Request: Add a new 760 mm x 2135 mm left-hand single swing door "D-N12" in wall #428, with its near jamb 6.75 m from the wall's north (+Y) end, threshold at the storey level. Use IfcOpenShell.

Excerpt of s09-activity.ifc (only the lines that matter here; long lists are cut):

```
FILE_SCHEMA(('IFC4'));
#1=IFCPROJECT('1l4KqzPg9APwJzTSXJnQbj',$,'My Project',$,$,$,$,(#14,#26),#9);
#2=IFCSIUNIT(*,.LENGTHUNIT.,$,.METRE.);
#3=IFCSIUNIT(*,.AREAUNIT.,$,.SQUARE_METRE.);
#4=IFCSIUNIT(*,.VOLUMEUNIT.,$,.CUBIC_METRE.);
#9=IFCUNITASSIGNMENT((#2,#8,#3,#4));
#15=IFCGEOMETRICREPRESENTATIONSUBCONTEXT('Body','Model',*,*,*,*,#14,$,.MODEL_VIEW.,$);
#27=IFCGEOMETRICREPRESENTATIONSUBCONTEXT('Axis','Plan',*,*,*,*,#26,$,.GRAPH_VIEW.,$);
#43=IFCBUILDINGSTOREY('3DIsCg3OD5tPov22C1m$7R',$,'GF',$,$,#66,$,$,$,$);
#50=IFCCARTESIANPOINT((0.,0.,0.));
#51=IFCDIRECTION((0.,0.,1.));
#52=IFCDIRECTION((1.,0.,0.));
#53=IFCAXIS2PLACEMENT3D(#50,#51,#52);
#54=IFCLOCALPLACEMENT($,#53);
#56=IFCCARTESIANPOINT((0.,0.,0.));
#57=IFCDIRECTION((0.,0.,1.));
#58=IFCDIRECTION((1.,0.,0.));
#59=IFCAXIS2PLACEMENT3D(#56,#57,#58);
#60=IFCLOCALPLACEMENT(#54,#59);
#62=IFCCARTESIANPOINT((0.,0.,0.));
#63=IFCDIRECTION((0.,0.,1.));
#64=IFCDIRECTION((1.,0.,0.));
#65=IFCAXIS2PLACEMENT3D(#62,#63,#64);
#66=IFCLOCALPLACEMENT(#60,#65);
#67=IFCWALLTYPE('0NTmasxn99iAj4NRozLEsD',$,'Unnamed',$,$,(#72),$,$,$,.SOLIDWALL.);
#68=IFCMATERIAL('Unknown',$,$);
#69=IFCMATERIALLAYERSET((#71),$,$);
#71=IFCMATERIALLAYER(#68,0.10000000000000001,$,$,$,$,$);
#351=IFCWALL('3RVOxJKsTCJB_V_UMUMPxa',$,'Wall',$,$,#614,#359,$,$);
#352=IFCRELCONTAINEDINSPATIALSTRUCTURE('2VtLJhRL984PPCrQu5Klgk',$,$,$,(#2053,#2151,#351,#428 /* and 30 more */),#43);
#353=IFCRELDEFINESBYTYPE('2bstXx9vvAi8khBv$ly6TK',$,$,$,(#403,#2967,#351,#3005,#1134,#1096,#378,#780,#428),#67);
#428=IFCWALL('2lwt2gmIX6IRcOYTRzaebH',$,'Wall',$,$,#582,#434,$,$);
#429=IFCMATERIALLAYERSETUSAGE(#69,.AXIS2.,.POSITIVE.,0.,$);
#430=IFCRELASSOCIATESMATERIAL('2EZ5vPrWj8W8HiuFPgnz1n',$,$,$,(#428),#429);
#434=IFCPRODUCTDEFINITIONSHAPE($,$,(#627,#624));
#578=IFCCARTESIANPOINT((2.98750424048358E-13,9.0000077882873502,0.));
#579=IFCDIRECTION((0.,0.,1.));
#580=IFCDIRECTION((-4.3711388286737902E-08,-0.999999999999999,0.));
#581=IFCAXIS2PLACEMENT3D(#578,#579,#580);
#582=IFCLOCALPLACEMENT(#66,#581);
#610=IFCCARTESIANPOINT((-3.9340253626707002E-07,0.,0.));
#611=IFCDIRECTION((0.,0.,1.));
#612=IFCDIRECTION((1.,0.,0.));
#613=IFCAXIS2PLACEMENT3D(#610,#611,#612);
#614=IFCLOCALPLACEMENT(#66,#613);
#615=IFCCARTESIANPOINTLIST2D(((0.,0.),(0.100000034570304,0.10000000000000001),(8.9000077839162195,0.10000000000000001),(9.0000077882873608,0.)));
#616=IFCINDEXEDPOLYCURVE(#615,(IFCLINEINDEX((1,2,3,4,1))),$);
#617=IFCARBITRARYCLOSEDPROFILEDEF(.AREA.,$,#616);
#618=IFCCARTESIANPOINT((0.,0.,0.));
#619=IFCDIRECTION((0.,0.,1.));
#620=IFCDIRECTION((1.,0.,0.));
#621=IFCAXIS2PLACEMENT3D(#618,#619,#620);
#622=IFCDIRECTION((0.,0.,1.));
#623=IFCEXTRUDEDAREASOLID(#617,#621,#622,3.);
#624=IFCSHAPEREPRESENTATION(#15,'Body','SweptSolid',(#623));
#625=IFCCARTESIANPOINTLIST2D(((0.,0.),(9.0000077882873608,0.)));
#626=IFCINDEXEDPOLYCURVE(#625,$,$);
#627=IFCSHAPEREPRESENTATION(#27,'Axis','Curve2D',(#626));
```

```python
import numpy as np
import ifcopenshell
import ifcopenshell.api.feature
import ifcopenshell.api.geometry
import ifcopenshell.api.root
import ifcopenshell.api.spatial
import ifcopenshell.geom
import ifcopenshell.util.element
import ifcopenshell.util.placement
import ifcopenshell.util.representation
import ifcopenshell.util.shape
import ifcopenshell.util.unit

model = ifcopenshell.open("s09-activity.ifc")
unit_scale = ifcopenshell.util.unit.calculate_unit_scale(model)
settings = ifcopenshell.geom.settings()


def volume(element):
    """Net volume in cubic metres, openings subtracted."""
    shape = ifcopenshell.geom.create_shape(settings, element)
    return ifcopenshell.util.shape.get_volume(shape.geometry)


wall = model.by_guid("2lwt2gmIX6IRcOYTRzaebH")
storey = ifcopenshell.util.element.get_container(wall, ifc_class="IfcBuildingStorey")
context = ifcopenshell.util.representation.get_context(model, "Model", "Body", "MODEL_VIEW")
before = volume(wall)

width, height, from_end, sill = 0.76, 2.135, 6.75, 0.0  # metres

# The wall runs along its own X axis, and the end named is its -X end.
wall_shape = ifcopenshell.geom.create_shape(settings, wall)
x, y, z = ifcopenshell.util.shape.get_vertices(wall_shape.geometry).T
start = x.min() + from_end
face, thickness = float(y.min()), float(y.max() - y.min())
wall_matrix = ifcopenshell.util.placement.get_local_placement(wall.ObjectPlacement)
level = ifcopenshell.util.placement.get_local_placement(storey.ObjectPlacement)[2, 3]


def in_wall(x, y):
    """Placement at x, y metres in the wall's axes, at sill height."""
    matrix = wall_matrix.copy()
    matrix[:, 3] = wall_matrix @ np.array([x / unit_scale, y / unit_scale, 0.0, 1.0])
    matrix[2, 3] = level + sill / unit_scale
    return matrix


# Opening: a box that overshoots both wall faces by 50 mm.
opening = ifcopenshell.api.root.create_entity(model, ifc_class="IfcOpeningElement", predefined_type="OPENING")
box = ifcopenshell.api.geometry.add_wall_representation(
    model, context=context, length=width, height=height, thickness=thickness + 0.1
)
ifcopenshell.api.geometry.assign_representation(model, product=opening, representation=box)
ifcopenshell.api.geometry.edit_object_placement(model, product=opening, matrix=in_wall(start, face - 0.05), is_si=False)
ifcopenshell.api.feature.add_feature(model, feature=opening, element=wall)

door = ifcopenshell.api.root.create_entity(model, ifc_class="IfcDoor", name="D-N12", predefined_type="DOOR")
door.OverallWidth, door.OverallHeight = width / unit_scale, height / unit_scale
door.OperationType = "SINGLE_SWING_LEFT"
body = ifcopenshell.api.geometry.add_door_representation(
    model,
    context=context,
    overall_width=door.OverallWidth,
    overall_height=door.OverallHeight,
    operation_type="SINGLE_SWING_LEFT",
    lining_properties={"LiningDepth": thickness / unit_scale, "ThresholdDepth": thickness / unit_scale},
)
ifcopenshell.api.geometry.assign_representation(model, product=door, representation=body)
ifcopenshell.api.spatial.assign_container(model, products=[door], relating_structure=storey)
ifcopenshell.api.feature.add_filling(model, opening=opening, element=door)

# The lining spans the wall, so the door starts at the wall face.
ifcopenshell.api.geometry.edit_object_placement(model, product=door, matrix=in_wall(start, face), is_si=False)

after = volume(wall)

print(f"wall volume {before:.3f} -> {after:.3f} m3")

model.write("s09-activity_updated.ifc")
```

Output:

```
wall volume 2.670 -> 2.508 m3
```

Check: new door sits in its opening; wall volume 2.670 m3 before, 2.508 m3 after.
